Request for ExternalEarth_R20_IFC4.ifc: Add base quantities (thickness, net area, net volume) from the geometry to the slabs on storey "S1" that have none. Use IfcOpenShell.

First a look at what the model holds.

```python
import ifcopenshell
import ifcopenshell.util.element
import ifcopenshell.util.unit

model = ifcopenshell.open("ExternalEarth_R20_IFC4.ifc")
print(model.schema)
for unit_type in ("LENGTHUNIT", "AREAUNIT", "VOLUMEUNIT"):
    print(unit_type, ifcopenshell.util.unit.calculate_unit_scale(model, unit_type))
storey = next(s for s in model.by_type("IfcBuildingStorey") if s.Name == "S1")
slabs = [e for e in ifcopenshell.util.element.get_decomposition(storey) if e.is_a("IfcSlab")]
for e in sorted(slabs, key=lambda e: e.id()):
    print(e.id(), e.is_a(), e.Name, list(ifcopenshell.util.element.get_psets(e, qtos_only=True)), sep=" | ")
```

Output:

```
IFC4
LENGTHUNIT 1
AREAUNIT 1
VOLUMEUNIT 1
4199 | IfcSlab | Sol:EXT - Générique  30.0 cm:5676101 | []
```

```python
import ifcopenshell
import ifcopenshell.api.pset
import ifcopenshell.geom
import ifcopenshell.util.element
import ifcopenshell.util.shape
import ifcopenshell.util.unit

model = ifcopenshell.open("ExternalEarth_R20_IFC4.ifc")
unit_scale = ifcopenshell.util.unit.calculate_unit_scale(model)
area_scale = ifcopenshell.util.unit.calculate_unit_scale(model, "AREAUNIT")
volume_scale = ifcopenshell.util.unit.calculate_unit_scale(model, "VOLUMEUNIT")
settings = ifcopenshell.geom.settings()

storey = next(s for s in model.by_type("IfcBuildingStorey") if s.Name == "S1")
slabs = [e for e in ifcopenshell.util.element.get_decomposition(storey) if e.is_a("IfcSlab")]

for e in sorted(slabs, key=lambda e: e.id()):
    if ifcopenshell.util.element.get_psets(e, qtos_only=True, should_inherit=False):
        continue
    # Geometry comes back in metres, in the element's own axes.
    shape = ifcopenshell.geom.create_shape(settings, e)
    values = {
        "Width": ifcopenshell.util.shape.get_z(shape.geometry) / unit_scale,
        "NetArea": ifcopenshell.util.shape.get_footprint_area(shape.geometry) / area_scale,
        "NetVolume": ifcopenshell.util.shape.get_volume(shape.geometry) / volume_scale,
    }
    qto = ifcopenshell.api.pset.add_qto(model, product=e, name="Qto_SlabBaseQuantities")
    ifcopenshell.api.pset.edit_qto(model, qto=qto, properties=values)
    print(e.id(), {k: round(v, 3) for k, v in values.items()})

model.write("ExternalEarth_R20_IFC4_rev.ifc")
```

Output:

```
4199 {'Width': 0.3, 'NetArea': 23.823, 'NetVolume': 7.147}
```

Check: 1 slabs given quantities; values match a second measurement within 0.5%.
